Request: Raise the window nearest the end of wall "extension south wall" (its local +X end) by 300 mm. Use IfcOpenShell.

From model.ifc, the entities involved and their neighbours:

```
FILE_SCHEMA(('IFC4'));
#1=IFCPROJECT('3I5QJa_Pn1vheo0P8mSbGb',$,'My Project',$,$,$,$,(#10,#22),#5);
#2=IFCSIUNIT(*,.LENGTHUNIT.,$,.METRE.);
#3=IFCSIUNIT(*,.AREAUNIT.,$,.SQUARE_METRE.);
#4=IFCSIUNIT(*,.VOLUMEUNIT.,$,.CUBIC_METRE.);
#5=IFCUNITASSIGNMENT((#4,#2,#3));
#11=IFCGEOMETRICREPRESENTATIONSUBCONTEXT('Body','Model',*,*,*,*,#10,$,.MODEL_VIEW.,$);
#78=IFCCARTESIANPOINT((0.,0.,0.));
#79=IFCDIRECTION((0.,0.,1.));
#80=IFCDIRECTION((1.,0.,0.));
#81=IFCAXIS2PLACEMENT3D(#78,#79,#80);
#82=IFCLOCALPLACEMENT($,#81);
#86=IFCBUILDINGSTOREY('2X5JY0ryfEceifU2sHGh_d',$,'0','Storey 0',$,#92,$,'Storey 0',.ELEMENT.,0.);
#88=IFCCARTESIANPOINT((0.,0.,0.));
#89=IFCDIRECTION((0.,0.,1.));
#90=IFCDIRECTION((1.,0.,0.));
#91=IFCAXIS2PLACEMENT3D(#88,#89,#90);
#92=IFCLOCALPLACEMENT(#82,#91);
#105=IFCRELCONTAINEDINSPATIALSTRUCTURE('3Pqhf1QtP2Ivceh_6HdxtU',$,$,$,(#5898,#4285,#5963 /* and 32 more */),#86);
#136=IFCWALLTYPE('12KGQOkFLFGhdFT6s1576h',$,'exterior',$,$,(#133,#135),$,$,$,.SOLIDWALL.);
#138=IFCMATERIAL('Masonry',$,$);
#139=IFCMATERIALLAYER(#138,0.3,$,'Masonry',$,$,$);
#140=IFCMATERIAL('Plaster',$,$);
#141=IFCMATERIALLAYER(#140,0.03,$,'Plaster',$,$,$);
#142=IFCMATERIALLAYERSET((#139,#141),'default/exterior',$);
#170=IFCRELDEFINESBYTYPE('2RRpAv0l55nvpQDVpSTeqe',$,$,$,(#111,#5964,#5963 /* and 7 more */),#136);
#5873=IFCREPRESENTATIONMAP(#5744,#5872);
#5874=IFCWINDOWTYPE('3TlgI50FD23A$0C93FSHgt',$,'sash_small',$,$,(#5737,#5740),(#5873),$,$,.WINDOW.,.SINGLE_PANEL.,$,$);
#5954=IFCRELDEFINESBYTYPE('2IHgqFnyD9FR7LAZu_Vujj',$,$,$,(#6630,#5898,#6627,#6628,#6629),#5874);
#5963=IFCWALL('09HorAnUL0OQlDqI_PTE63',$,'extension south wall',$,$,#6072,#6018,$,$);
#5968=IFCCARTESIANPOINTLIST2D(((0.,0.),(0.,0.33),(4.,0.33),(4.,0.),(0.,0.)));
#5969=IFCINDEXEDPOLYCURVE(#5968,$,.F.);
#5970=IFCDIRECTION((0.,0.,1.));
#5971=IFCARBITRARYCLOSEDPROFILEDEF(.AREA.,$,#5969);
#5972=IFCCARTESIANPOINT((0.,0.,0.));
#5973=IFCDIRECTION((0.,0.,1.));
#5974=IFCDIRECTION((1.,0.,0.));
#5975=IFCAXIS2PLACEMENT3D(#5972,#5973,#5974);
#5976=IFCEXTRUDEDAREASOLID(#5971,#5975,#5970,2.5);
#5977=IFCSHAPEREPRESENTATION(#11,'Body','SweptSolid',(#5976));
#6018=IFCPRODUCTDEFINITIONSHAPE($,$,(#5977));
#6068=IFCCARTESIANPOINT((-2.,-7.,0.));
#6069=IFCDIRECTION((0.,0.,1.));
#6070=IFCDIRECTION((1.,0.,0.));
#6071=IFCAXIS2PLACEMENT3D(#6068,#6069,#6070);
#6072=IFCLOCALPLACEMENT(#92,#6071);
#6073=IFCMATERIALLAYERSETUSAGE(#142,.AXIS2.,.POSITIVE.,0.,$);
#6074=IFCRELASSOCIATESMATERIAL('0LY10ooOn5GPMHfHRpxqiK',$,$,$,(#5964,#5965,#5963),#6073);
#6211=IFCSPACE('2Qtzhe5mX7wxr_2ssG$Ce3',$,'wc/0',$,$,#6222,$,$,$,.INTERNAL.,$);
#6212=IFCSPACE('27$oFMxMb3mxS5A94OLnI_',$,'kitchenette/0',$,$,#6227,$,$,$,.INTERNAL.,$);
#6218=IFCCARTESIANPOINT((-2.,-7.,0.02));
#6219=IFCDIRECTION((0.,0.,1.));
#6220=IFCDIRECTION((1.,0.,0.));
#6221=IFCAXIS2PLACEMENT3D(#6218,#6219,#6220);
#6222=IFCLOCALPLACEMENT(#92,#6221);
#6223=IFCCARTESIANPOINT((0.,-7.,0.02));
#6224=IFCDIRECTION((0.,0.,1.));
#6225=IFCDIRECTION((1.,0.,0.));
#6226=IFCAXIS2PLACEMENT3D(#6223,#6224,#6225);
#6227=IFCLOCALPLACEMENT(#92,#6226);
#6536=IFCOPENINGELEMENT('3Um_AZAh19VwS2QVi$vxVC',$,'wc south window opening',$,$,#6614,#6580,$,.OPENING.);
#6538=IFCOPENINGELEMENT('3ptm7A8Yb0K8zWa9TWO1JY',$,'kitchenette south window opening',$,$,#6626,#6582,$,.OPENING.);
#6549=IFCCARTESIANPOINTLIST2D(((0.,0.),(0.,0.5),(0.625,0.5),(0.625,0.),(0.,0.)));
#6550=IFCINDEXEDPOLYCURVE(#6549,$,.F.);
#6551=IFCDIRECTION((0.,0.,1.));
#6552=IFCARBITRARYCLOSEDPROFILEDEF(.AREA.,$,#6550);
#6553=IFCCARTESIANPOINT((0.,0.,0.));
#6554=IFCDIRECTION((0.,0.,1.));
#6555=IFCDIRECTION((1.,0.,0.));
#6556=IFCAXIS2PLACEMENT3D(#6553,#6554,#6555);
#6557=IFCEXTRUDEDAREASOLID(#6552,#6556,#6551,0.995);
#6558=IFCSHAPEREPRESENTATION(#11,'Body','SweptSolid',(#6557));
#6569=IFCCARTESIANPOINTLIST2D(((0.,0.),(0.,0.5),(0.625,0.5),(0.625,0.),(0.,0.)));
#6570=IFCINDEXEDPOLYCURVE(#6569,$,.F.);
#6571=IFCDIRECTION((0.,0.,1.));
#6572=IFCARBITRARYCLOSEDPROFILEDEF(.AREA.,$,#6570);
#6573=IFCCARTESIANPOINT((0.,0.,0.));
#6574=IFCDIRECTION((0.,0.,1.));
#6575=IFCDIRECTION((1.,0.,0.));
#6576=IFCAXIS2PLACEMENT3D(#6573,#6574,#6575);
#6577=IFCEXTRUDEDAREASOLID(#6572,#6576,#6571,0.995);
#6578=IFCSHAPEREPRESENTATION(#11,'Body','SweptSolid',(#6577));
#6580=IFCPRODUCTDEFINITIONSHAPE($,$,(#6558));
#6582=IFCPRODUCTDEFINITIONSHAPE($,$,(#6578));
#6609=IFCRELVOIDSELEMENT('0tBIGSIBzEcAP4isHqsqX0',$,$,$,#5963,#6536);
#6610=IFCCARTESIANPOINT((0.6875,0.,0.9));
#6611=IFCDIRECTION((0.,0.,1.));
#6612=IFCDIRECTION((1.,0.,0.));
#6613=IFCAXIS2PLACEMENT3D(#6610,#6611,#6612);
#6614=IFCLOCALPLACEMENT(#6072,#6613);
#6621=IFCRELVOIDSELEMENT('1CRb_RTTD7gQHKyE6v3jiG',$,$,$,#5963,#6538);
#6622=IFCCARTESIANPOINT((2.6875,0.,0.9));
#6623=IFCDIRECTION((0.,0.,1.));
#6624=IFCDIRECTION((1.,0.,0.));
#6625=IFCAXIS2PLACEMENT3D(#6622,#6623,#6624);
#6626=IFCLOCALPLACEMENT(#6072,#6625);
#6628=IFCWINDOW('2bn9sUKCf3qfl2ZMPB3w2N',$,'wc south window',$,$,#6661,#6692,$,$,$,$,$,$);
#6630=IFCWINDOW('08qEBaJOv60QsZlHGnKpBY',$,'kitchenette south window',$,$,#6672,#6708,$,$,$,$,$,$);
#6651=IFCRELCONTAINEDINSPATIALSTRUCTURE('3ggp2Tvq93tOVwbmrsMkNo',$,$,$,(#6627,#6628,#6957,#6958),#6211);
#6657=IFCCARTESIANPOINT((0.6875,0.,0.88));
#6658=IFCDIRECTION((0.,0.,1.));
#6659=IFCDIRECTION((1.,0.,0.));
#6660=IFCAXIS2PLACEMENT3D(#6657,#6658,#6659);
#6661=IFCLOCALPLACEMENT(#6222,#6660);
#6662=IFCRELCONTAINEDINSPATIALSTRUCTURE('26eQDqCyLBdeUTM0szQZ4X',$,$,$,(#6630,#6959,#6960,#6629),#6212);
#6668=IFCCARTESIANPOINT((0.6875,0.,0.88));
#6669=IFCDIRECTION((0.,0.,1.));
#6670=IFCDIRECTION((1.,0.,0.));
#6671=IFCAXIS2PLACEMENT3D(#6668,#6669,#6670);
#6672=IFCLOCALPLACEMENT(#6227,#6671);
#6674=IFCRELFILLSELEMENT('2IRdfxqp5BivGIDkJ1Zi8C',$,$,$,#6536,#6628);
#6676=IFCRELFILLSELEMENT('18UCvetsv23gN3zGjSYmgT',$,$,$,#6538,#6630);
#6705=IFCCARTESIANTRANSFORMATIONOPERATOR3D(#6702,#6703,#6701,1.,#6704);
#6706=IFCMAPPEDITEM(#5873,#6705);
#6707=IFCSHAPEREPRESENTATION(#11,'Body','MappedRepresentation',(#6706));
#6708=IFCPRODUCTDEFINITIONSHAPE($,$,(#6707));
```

```python
import numpy as np
import ifcopenshell
import ifcopenshell.api.geometry
import ifcopenshell.util.placement
import ifcopenshell.util.unit

model = ifcopenshell.open("model.ifc")
unit_scale = ifcopenshell.util.unit.calculate_unit_scale(model)

window = model.by_guid("08qEBaJOv60QsZlHGnKpBY")
opening = window.FillsVoids[0].RelatingOpeningElement
dz = 0.3

shift = np.array([0.0, 0.0, dz])
# The window is not placed relative to its opening, so move both.
for product in (opening, window):
    matrix = ifcopenshell.util.placement.get_local_placement(product.ObjectPlacement)
    matrix[:3, 3] += shift
    ifcopenshell.api.geometry.edit_object_placement(model, product=product, matrix=matrix, is_si=False)

print(f"moved by {dz * unit_scale:+.3f} m")

model.write("model_edited.ifc")
```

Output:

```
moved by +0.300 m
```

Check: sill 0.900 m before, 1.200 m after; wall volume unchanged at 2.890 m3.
